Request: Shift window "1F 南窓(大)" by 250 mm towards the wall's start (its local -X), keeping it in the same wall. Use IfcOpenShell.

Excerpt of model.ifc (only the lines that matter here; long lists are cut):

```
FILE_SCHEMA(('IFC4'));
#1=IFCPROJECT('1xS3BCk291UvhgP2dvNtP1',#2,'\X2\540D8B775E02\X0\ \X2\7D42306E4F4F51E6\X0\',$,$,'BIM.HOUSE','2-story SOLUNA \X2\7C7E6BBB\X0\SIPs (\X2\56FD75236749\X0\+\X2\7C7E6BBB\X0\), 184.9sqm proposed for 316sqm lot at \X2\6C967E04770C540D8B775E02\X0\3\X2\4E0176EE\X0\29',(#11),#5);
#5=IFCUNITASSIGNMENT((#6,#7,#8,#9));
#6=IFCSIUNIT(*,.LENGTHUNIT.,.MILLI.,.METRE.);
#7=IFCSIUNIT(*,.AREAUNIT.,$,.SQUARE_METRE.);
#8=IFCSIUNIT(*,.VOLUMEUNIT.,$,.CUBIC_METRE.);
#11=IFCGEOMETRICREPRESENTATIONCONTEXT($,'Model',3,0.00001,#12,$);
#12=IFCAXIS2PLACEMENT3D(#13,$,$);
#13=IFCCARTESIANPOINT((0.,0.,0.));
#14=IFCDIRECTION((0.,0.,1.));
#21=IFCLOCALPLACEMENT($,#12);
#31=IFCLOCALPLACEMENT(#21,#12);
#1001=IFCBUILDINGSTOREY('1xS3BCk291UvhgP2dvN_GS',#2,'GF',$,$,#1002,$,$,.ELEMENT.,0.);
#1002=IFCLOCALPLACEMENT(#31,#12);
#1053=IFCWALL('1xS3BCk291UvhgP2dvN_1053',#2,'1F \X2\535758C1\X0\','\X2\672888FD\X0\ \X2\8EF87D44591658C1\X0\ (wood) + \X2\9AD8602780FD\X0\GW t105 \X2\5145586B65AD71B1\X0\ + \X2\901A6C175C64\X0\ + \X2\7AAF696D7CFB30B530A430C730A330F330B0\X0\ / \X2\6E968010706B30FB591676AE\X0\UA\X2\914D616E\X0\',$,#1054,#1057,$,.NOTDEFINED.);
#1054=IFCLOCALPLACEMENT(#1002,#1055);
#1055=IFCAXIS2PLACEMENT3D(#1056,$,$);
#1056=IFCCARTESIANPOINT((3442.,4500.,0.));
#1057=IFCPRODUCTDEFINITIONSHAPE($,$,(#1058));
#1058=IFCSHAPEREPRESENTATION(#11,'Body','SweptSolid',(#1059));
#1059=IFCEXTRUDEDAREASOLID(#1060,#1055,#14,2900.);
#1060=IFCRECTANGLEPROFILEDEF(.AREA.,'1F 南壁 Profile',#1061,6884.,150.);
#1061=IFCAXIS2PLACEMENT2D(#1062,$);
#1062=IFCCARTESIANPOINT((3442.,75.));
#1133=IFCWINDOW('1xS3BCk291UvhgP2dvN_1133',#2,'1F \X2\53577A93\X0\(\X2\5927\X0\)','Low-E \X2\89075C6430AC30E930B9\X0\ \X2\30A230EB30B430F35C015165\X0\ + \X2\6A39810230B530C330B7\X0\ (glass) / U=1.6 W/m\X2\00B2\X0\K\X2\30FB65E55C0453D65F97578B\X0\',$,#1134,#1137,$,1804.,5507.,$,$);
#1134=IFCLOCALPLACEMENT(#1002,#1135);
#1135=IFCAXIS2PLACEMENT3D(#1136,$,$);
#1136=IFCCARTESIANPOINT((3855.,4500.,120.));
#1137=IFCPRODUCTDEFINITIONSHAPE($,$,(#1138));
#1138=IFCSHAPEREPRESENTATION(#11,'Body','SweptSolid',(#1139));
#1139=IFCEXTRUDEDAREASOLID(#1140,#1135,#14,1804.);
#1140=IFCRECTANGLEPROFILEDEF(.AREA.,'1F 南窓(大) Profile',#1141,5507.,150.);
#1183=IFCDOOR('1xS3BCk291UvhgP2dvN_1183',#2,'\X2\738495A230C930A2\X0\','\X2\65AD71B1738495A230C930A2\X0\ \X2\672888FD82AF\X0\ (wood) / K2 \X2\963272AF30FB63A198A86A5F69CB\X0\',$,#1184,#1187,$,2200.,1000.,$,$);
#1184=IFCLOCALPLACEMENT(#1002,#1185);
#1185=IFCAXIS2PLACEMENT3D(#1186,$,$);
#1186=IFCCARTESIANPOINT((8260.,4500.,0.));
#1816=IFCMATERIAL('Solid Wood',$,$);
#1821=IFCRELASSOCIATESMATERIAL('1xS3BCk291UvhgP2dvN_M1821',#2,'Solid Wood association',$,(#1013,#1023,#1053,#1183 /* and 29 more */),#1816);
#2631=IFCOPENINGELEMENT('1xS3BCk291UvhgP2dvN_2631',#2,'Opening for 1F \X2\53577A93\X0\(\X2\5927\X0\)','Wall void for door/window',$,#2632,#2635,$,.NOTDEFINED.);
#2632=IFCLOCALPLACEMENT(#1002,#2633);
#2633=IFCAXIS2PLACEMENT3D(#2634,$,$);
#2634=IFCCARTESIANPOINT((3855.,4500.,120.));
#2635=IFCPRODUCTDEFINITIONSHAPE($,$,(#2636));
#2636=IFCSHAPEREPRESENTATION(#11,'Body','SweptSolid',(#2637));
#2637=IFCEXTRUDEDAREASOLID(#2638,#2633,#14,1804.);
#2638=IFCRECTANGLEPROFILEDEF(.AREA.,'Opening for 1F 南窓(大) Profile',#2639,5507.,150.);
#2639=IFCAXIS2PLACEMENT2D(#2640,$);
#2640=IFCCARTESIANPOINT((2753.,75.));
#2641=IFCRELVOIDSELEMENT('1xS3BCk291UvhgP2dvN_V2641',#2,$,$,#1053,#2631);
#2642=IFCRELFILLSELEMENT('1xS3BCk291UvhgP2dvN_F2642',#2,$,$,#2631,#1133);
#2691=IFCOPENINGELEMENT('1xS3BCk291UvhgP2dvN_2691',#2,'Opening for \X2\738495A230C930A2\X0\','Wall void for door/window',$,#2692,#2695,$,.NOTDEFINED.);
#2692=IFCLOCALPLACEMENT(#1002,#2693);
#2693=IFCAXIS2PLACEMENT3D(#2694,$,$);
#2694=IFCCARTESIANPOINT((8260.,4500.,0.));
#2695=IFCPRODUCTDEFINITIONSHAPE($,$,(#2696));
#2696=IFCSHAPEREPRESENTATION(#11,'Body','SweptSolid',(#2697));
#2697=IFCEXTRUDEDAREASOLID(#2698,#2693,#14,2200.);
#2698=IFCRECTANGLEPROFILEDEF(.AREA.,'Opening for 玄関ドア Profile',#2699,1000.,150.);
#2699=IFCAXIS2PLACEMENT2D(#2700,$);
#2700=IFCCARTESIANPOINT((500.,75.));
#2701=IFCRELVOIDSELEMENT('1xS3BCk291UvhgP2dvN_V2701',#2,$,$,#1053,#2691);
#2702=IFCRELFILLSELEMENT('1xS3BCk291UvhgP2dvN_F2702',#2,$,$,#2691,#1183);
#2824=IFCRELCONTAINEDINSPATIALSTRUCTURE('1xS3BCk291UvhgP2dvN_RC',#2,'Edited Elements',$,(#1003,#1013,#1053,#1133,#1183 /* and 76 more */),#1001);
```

```python
import ifcopenshell
import ifcopenshell.api.geometry
import ifcopenshell.util.placement
import ifcopenshell.util.unit

model = ifcopenshell.open("model.ifc")
unit_scale = ifcopenshell.util.unit.calculate_unit_scale(model)

window = model.by_guid("1xS3BCk291UvhgP2dvN_1133")
opening = window.FillsVoids[0].RelatingOpeningElement
wall = opening.VoidsElements[0].RelatingBuildingElement

wall_matrix = ifcopenshell.util.placement.get_local_placement(wall.ObjectPlacement)
shift = wall_matrix[:3, 0] * -0.25 / unit_scale
before = ifcopenshell.util.placement.get_local_placement(window.ObjectPlacement)[:3, 3].copy()

# The window is not placed relative to its opening, so move both.
for product in (opening, window):
    matrix = ifcopenshell.util.placement.get_local_placement(product.ObjectPlacement)
    matrix[:3, 3] += shift
    ifcopenshell.api.geometry.edit_object_placement(model, product=product, matrix=matrix, is_si=False)

after = ifcopenshell.util.placement.get_local_placement(window.ObjectPlacement)[:3, 3]
print("window moved by", (after - before).round(3) + 0.0)

model.write("model_rev.ifc")
```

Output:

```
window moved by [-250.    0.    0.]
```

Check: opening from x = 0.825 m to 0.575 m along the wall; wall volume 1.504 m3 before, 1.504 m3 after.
